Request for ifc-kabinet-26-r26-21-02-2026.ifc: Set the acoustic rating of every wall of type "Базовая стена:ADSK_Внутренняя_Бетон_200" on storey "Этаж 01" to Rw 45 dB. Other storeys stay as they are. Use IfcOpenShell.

First a look at what the model holds.

```python
import ifcopenshell
import ifcopenshell.util.element

model = ifcopenshell.open("ifc-kabinet-26-r26-21-02-2026.ifc")
print(model.schema)
storey = next(s for s in model.by_type("IfcBuildingStorey") if s.Name == "Этаж 01")
walls = [e for e in ifcopenshell.util.element.get_decomposition(storey) if e.is_a("IfcWall")]
seen = {}
for e in walls:
    element_type = ifcopenshell.util.element.get_type(e)
    key = (element_type.Name if element_type != e and element_type else None, ifcopenshell.util.element.get_pset(e, "Pset_WallCommon", "AcousticRating"))
    seen[key] = seen.get(key, 0) + 1
for (name, value), count in sorted(seen.items(), key=str):
    print(count, "x", name, "|", value)
```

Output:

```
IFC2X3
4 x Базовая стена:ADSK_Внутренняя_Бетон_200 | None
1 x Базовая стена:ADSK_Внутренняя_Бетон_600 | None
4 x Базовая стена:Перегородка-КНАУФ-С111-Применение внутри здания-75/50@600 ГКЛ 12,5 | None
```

```python
import ifcopenshell
import ifcopenshell.api.pset
import ifcopenshell.util.element

model = ifcopenshell.open("ifc-kabinet-26-r26-21-02-2026.ifc")

storey = next(s for s in model.by_type("IfcBuildingStorey") if s.Name == "Этаж 01")
walls = [e for e in ifcopenshell.util.element.get_decomposition(storey) if e.is_a("IfcWall")]

count = 0
for e in walls:
    element_type = ifcopenshell.util.element.get_type(e)
    if element_type in (None, e) or element_type.Name != "Базовая стена:ADSK_Внутренняя_Бетон_200":
        continue
    # add_pset returns the element's existing set when there is one.
    pset = ifcopenshell.api.pset.add_pset(model, product=e, name="Pset_WallCommon")
    ifcopenshell.api.pset.edit_pset(model, pset=pset, properties={"AcousticRating": "Rw 45 dB"})
    count += 1

print(count, "walls updated")

model.write("ifc-kabinet-26-r26-21-02-2026_v2.ifc")
```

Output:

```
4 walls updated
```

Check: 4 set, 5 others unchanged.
